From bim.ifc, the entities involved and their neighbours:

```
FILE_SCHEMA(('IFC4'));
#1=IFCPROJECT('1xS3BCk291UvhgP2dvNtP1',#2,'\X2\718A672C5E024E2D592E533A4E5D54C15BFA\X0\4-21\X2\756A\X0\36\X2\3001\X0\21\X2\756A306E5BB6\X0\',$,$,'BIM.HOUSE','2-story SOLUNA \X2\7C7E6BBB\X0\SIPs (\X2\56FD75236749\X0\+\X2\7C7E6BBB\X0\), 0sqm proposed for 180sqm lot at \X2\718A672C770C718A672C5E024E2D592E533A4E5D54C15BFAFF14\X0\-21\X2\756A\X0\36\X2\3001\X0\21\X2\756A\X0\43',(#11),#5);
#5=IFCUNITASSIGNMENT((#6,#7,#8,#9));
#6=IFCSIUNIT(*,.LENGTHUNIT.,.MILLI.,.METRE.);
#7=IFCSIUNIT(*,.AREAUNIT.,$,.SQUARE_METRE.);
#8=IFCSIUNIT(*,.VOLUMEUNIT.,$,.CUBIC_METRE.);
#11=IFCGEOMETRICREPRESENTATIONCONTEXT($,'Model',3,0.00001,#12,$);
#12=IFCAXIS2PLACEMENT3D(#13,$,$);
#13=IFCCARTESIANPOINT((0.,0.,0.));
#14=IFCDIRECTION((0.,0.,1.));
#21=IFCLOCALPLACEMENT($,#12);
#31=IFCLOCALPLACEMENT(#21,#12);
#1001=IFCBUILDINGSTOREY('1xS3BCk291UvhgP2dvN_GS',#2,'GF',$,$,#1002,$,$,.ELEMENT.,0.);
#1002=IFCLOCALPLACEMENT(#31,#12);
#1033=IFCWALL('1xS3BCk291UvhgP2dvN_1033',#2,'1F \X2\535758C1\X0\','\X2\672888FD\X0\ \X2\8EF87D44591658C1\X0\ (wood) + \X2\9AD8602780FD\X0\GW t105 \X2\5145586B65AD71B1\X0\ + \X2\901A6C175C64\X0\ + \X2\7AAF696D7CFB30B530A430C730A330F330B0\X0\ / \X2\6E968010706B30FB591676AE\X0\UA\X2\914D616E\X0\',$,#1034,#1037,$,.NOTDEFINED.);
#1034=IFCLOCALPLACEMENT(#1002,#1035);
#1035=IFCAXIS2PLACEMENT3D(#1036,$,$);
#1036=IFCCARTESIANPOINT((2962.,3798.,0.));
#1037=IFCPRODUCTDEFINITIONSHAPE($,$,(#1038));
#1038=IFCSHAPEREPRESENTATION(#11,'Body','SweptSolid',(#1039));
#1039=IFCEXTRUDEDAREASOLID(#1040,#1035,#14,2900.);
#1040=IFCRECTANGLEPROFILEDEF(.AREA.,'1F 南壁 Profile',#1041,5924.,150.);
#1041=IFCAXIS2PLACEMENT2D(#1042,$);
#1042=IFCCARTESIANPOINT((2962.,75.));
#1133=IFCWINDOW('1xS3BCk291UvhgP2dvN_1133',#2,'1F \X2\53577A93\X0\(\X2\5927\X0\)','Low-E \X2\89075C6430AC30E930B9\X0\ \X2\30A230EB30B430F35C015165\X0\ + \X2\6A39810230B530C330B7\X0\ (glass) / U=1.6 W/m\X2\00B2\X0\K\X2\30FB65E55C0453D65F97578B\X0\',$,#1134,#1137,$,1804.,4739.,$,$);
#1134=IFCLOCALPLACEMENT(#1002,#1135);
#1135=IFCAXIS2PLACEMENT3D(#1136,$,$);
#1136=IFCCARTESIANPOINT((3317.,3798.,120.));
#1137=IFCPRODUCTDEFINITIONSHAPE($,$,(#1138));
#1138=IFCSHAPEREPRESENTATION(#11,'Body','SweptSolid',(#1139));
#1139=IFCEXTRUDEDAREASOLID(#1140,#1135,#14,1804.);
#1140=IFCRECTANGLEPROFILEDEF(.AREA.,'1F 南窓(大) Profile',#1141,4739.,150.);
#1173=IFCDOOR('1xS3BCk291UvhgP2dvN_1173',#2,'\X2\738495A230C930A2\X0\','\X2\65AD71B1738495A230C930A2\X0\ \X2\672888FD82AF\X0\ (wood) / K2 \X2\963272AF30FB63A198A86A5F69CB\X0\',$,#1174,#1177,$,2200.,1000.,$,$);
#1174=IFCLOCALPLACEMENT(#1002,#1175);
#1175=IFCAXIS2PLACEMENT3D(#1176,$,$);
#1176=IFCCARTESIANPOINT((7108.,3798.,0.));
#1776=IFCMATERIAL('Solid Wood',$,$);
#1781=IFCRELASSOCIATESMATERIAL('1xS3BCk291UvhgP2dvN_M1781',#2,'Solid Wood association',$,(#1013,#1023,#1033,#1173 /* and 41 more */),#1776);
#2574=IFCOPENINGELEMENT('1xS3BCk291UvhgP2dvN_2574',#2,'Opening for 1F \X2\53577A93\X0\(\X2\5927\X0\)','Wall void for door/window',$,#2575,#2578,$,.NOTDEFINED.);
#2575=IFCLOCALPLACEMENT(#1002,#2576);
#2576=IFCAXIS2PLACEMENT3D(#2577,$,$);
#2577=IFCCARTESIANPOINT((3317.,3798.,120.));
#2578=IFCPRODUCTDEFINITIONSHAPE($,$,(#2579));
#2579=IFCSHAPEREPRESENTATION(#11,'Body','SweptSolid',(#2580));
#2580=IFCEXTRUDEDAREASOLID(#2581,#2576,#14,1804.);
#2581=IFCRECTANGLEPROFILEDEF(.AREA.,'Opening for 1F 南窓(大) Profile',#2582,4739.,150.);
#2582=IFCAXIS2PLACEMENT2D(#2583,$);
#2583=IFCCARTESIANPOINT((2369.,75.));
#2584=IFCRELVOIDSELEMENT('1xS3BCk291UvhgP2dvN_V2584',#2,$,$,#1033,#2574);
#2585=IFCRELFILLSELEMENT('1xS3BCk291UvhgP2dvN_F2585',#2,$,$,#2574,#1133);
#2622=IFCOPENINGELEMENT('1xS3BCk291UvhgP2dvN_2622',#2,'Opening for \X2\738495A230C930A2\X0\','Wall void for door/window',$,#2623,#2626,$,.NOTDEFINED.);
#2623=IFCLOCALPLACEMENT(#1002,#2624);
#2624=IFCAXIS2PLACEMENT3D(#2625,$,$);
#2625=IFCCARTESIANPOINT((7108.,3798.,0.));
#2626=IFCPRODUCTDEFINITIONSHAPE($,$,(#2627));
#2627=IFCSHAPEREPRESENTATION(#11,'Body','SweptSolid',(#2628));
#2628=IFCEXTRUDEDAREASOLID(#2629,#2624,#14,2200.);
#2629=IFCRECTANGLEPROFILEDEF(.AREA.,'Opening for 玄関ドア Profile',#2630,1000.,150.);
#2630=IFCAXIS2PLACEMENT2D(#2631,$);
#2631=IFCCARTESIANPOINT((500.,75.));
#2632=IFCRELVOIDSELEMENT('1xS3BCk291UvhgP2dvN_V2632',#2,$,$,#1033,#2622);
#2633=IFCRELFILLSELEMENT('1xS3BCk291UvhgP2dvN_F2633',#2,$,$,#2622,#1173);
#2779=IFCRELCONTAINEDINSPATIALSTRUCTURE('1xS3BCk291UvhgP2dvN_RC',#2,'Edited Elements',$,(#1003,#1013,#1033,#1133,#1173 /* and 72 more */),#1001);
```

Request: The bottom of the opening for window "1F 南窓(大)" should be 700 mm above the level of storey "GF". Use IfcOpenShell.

```python
import numpy as np
import ifcopenshell
import ifcopenshell.api.geometry
import ifcopenshell.geom
import ifcopenshell.util.element
import ifcopenshell.util.placement
import ifcopenshell.util.shape
import ifcopenshell.util.unit

model = ifcopenshell.open("bim.ifc")
unit_scale = ifcopenshell.util.unit.calculate_unit_scale(model)

window = model.by_guid("1xS3BCk291UvhgP2dvN_1133")
opening = window.FillsVoids[0].RelatingOpeningElement
storey = ifcopenshell.util.element.get_container(window, ifc_class="IfcBuildingStorey")
level = ifcopenshell.util.placement.get_local_placement(storey.ObjectPlacement)[2, 3]

# The opening's origin need not be at the sill, so measure its lowest point.
shape = ifcopenshell.geom.create_shape(ifcopenshell.geom.settings(), opening)
bottom = ifcopenshell.util.shape.get_shape_bottom_elevation(shape, shape.geometry) / unit_scale
dz = level + 0.7 / unit_scale - bottom

shift = np.array([0.0, 0.0, dz])
# The window is not placed relative to its opening, so move both.
for product in (opening, window):
    matrix = ifcopenshell.util.placement.get_local_placement(product.ObjectPlacement)
    matrix[:3, 3] += shift
    ifcopenshell.api.geometry.edit_object_placement(model, product=product, matrix=matrix, is_si=False)

print(f"moved by {dz * unit_scale:+.3f} m")

model.write("bim_edited.ifc")
```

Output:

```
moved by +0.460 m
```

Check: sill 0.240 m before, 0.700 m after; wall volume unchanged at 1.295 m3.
